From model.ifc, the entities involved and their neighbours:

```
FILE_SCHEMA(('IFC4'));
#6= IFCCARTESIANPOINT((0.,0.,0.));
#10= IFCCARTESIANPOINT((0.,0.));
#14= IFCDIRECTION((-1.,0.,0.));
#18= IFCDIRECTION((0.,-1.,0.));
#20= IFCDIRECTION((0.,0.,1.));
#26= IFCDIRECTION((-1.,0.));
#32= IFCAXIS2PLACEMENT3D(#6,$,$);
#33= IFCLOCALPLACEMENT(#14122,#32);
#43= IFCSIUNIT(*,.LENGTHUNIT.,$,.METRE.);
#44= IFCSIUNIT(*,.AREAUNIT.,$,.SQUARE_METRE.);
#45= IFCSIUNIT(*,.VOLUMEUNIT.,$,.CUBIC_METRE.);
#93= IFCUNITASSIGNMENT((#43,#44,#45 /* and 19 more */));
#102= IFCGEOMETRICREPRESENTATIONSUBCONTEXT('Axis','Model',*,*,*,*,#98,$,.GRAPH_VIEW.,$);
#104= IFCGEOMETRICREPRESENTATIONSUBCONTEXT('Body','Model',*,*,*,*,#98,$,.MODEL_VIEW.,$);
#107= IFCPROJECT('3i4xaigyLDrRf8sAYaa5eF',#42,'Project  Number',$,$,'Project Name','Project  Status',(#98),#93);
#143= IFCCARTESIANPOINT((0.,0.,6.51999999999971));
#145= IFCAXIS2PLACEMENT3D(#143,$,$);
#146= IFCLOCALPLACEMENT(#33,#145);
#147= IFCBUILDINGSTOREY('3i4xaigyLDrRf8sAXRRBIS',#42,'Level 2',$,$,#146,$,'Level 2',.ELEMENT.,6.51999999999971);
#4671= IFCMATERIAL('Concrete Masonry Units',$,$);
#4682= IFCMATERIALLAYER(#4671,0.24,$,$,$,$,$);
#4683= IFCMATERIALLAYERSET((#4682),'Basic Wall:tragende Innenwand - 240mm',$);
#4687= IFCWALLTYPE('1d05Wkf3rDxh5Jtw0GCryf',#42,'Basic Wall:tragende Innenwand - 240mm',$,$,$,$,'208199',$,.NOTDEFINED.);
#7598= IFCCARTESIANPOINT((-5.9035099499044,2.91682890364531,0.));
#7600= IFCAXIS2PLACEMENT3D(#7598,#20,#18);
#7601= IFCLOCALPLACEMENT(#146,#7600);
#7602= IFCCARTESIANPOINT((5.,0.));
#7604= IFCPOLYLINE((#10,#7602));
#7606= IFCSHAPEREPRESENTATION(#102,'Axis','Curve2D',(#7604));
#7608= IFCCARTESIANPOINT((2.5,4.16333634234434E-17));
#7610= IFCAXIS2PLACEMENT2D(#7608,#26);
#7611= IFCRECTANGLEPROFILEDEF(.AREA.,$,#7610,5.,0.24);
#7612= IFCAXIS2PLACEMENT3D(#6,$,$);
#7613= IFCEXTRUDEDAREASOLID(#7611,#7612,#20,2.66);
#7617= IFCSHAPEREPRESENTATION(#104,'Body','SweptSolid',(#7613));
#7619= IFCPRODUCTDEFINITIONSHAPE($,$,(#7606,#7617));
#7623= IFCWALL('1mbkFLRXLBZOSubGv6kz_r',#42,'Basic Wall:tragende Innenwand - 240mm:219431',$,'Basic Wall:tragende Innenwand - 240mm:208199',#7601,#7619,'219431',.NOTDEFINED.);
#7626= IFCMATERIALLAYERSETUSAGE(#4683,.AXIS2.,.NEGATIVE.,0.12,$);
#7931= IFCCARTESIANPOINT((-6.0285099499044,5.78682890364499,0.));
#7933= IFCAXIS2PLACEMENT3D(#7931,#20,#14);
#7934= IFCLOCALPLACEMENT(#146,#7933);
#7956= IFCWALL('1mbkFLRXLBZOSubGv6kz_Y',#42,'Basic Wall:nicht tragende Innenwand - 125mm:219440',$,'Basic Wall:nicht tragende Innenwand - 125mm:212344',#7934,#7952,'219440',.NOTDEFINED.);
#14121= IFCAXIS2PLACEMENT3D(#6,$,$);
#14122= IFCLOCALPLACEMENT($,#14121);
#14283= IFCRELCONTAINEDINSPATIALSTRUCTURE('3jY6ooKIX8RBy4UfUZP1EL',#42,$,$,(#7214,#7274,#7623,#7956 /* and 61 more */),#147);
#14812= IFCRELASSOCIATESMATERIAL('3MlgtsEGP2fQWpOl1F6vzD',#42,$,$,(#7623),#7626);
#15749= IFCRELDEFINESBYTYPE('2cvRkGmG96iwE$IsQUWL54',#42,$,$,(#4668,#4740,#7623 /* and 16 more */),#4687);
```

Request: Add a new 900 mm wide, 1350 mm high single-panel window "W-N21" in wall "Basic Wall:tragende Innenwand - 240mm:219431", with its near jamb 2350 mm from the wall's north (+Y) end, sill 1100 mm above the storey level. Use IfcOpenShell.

```python
import numpy as np
import ifcopenshell
import ifcopenshell.api.feature
import ifcopenshell.api.geometry
import ifcopenshell.api.root
import ifcopenshell.api.spatial
import ifcopenshell.geom
import ifcopenshell.util.element
import ifcopenshell.util.placement
import ifcopenshell.util.representation
import ifcopenshell.util.shape
import ifcopenshell.util.unit

model = ifcopenshell.open("model.ifc")
unit_scale = ifcopenshell.util.unit.calculate_unit_scale(model)
settings = ifcopenshell.geom.settings()


def volume(element):
    """Net volume in cubic metres, openings subtracted."""
    shape = ifcopenshell.geom.create_shape(settings, element)
    return ifcopenshell.util.shape.get_volume(shape.geometry)


wall = model.by_guid("1mbkFLRXLBZOSubGv6kz_r")
storey = ifcopenshell.util.element.get_container(wall, ifc_class="IfcBuildingStorey")
context = ifcopenshell.util.representation.get_context(model, "Model", "Body", "MODEL_VIEW")
before = volume(wall)

width, height, from_end, sill = 0.9, 1.35, 2.35, 1.1  # metres

# The wall runs along its own X axis, and the end named is its -X end.
wall_shape = ifcopenshell.geom.create_shape(settings, wall)
x, y, z = ifcopenshell.util.shape.get_vertices(wall_shape.geometry).T
start = x.min() + from_end
face, thickness = float(y.min()), float(y.max() - y.min())
wall_matrix = ifcopenshell.util.placement.get_local_placement(wall.ObjectPlacement)
level = ifcopenshell.util.placement.get_local_placement(storey.ObjectPlacement)[2, 3]


def in_wall(x, y):
    """Placement at x, y metres in the wall's axes, at sill height."""
    matrix = wall_matrix.copy()
    matrix[:, 3] = wall_matrix @ np.array([x / unit_scale, y / unit_scale, 0.0, 1.0])
    matrix[2, 3] = level + sill / unit_scale
    return matrix


# Opening: a box that overshoots both wall faces by 50 mm.
opening = ifcopenshell.api.root.create_entity(model, ifc_class="IfcOpeningElement", predefined_type="OPENING")
box = ifcopenshell.api.geometry.add_wall_representation(
    model, context=context, length=width, height=height, thickness=thickness + 0.1
)
ifcopenshell.api.geometry.assign_representation(model, product=opening, representation=box)
ifcopenshell.api.geometry.edit_object_placement(model, product=opening, matrix=in_wall(start, face - 0.05), is_si=False)
ifcopenshell.api.feature.add_feature(model, feature=opening, element=wall)

window = ifcopenshell.api.root.create_entity(model, ifc_class="IfcWindow", name="W-N21", predefined_type="WINDOW")
window.OverallWidth, window.OverallHeight = width / unit_scale, height / unit_scale
window.PartitioningType = "SINGLE_PANEL"
body = ifcopenshell.api.geometry.add_window_representation(
    model,
    context=context,
    overall_width=window.OverallWidth,
    overall_height=window.OverallHeight,
    partition_type="SINGLE_PANEL",
)
ifcopenshell.api.geometry.assign_representation(model, product=window, representation=body)
ifcopenshell.api.spatial.assign_container(model, products=[window], relating_structure=storey)
ifcopenshell.api.feature.add_filling(model, opening=opening, element=window)

# Centre the window in the wall's thickness.
ifcopenshell.api.geometry.edit_object_placement(model, product=window, matrix=in_wall(start, face), is_si=False)
window_shape = ifcopenshell.geom.create_shape(settings, window)
depth = ifcopenshell.util.shape.get_vertices(window_shape.geometry)[:, 1]
offset = face + thickness / 2 - (depth.min() + depth.max()) / 2
ifcopenshell.api.geometry.edit_object_placement(model, product=window, matrix=in_wall(start, offset), is_si=False)

after = volume(wall)

print(f"wall volume {before:.3f} -> {after:.3f} m3")

model.write("model_updated.ifc")
```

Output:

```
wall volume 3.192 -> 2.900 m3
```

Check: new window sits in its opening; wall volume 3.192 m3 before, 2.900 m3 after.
